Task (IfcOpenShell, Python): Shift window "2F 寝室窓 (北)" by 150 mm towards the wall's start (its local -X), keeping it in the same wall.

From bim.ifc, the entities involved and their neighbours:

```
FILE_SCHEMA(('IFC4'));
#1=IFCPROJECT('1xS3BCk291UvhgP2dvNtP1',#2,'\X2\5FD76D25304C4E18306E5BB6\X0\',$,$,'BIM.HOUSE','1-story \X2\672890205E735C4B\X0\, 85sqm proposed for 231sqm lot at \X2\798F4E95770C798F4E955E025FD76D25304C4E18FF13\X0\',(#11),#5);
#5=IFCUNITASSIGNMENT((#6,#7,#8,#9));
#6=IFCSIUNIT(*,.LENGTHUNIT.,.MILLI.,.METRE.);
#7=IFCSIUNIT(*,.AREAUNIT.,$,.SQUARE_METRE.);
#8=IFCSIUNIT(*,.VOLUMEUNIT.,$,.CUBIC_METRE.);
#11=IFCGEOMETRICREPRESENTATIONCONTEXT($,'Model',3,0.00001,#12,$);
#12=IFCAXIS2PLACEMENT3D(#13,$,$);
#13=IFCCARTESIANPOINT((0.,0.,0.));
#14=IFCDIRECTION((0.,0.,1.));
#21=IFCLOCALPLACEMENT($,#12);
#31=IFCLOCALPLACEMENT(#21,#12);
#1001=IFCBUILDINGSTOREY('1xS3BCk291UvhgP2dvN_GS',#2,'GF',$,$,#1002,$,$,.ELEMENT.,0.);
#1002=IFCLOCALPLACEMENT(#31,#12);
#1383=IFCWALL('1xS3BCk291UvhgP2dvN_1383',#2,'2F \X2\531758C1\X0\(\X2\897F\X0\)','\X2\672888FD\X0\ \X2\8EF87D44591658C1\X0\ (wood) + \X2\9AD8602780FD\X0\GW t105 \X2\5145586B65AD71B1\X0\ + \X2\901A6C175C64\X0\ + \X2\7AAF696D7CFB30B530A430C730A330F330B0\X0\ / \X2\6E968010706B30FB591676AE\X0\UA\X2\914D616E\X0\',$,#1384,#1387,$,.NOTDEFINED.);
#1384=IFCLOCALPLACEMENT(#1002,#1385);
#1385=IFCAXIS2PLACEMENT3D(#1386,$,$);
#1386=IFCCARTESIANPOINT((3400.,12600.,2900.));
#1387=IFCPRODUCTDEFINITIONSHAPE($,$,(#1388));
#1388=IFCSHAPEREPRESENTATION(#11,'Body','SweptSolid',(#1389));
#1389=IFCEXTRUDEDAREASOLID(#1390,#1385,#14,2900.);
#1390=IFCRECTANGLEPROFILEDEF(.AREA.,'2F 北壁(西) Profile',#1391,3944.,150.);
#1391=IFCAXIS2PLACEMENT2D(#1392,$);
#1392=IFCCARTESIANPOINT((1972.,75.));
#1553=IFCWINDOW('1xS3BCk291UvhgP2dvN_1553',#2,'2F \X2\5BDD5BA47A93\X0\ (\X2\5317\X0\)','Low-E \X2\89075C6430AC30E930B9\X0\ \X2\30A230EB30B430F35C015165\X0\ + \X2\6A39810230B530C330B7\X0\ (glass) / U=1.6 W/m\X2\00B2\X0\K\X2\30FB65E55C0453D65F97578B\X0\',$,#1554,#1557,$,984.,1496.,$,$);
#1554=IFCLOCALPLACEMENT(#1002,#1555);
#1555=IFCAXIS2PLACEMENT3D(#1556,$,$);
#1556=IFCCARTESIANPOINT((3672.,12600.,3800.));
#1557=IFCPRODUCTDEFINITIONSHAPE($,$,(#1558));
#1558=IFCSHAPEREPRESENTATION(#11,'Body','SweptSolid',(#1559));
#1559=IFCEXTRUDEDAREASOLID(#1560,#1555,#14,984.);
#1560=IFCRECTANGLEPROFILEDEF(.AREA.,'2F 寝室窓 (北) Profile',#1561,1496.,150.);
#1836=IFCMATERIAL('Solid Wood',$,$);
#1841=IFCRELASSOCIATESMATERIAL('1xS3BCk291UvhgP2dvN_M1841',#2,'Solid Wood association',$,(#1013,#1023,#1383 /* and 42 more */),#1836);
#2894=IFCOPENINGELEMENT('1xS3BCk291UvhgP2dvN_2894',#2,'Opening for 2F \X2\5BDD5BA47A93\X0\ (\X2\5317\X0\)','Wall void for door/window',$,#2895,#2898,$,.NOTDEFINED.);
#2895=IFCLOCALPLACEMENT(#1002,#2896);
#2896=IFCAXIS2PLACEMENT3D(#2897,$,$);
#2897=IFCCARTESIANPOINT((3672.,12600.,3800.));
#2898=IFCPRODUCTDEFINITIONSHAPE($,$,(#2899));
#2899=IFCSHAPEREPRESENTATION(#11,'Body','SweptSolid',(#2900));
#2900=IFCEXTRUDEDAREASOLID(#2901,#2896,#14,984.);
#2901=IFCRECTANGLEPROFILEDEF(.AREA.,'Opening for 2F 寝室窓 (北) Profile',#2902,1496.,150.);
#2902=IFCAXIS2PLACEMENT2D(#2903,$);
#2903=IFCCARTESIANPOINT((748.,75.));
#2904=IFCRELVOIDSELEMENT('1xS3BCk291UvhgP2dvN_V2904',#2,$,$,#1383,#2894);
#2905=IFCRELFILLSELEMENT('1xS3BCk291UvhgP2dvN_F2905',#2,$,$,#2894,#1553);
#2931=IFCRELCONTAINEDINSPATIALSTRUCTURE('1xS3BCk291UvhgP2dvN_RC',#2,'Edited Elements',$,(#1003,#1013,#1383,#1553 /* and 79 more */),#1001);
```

```python
import ifcopenshell
import ifcopenshell.api.geometry
import ifcopenshell.util.placement
import ifcopenshell.util.unit

model = ifcopenshell.open("bim.ifc")
unit_scale = ifcopenshell.util.unit.calculate_unit_scale(model)

window = model.by_guid("1xS3BCk291UvhgP2dvN_1553")
opening = window.FillsVoids[0].RelatingOpeningElement
wall = opening.VoidsElements[0].RelatingBuildingElement

wall_matrix = ifcopenshell.util.placement.get_local_placement(wall.ObjectPlacement)
shift = wall_matrix[:3, 0] * -0.15 / unit_scale
before = ifcopenshell.util.placement.get_local_placement(window.ObjectPlacement)[:3, 3].copy()

# The window is not placed relative to its opening, so move both.
for product in (opening, window):
    matrix = ifcopenshell.util.placement.get_local_placement(product.ObjectPlacement)
    matrix[:3, 3] += shift
    ifcopenshell.api.geometry.edit_object_placement(model, product=product, matrix=matrix, is_si=False)

after = ifcopenshell.util.placement.get_local_placement(window.ObjectPlacement)[:3, 3]
print("window moved by", (after - before).round(3) + 0.0)

model.write("bim_v2.ifc")
```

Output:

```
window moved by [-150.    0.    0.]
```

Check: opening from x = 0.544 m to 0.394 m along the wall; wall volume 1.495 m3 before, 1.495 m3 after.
